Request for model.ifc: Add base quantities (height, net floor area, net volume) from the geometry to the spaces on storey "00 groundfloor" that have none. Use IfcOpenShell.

First a look at what the model holds.

```python
import ifcopenshell
import ifcopenshell.util.element
import ifcopenshell.util.unit

model = ifcopenshell.open("model.ifc")
print(model.schema)
for unit_type in ("LENGTHUNIT", "AREAUNIT", "VOLUMEUNIT"):
    print(unit_type, ifcopenshell.util.unit.calculate_unit_scale(model, unit_type))
storey = next(s for s in model.by_type("IfcBuildingStorey") if s.Name == "00 groundfloor")
spaces = [e for e in ifcopenshell.util.element.get_decomposition(storey) if e.is_a("IfcSpace")]
for e in sorted(spaces, key=lambda e: e.id()):
    print(e.id(), e.is_a(), e.Name, list(ifcopenshell.util.element.get_psets(e, qtos_only=True)), sep=" | ")
```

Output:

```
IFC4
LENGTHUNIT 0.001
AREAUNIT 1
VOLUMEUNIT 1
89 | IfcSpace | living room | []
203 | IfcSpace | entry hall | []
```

```python
import ifcopenshell
import ifcopenshell.api.pset
import ifcopenshell.geom
import ifcopenshell.util.element
import ifcopenshell.util.shape
import ifcopenshell.util.unit

model = ifcopenshell.open("model.ifc")
unit_scale = ifcopenshell.util.unit.calculate_unit_scale(model)
area_scale = ifcopenshell.util.unit.calculate_unit_scale(model, "AREAUNIT")
volume_scale = ifcopenshell.util.unit.calculate_unit_scale(model, "VOLUMEUNIT")
settings = ifcopenshell.geom.settings()

storey = next(s for s in model.by_type("IfcBuildingStorey") if s.Name == "00 groundfloor")
spaces = [e for e in ifcopenshell.util.element.get_decomposition(storey) if e.is_a("IfcSpace")]

for e in sorted(spaces, key=lambda e: e.id()):
    if ifcopenshell.util.element.get_psets(e, qtos_only=True, should_inherit=False):
        continue
    # Geometry comes back in metres, in the element's own axes.
    shape = ifcopenshell.geom.create_shape(settings, e)
    values = {
        "Height": ifcopenshell.util.shape.get_z(shape.geometry) / unit_scale,
        "NetFloorArea": ifcopenshell.util.shape.get_footprint_area(shape.geometry) / area_scale,
        "NetVolume": ifcopenshell.util.shape.get_volume(shape.geometry) / volume_scale,
    }
    qto = ifcopenshell.api.pset.add_qto(model, product=e, name="Qto_SpaceBaseQuantities")
    ifcopenshell.api.pset.edit_qto(model, qto=qto, properties=values)
    print(e.id(), {k: round(v, 3) for k, v in values.items()})

model.write("model-out.ifc")
```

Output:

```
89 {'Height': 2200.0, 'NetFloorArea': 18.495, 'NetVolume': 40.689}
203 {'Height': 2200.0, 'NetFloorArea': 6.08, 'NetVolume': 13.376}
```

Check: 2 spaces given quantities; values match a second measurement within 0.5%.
